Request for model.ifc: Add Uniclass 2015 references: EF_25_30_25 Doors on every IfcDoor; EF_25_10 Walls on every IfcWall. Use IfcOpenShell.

First a look at what the model holds.

```python
import ifcopenshell

model = ifcopenshell.open("model.ifc")
print(model.schema)
print("classifications:", [c.Name for c in model.by_type("IfcClassification")])
for ifc_class in ("IfcDoor", "IfcRoof", "IfcStair", "IfcWall", "IfcWindow"):
    print(ifc_class, len(model.by_type(ifc_class)))
```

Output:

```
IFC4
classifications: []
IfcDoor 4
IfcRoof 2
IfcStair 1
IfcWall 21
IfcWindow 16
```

```python
import ifcopenshell
import ifcopenshell.api.classification

model = ifcopenshell.open("model.ifc")

system = ifcopenshell.api.classification.add_classification(model, classification="Uniclass 2015")

codes = {
    "IfcDoor": ("EF_25_30_25", "Doors"),
    "IfcWall": ("EF_25_10", "Walls"),
}
for ifc_class, (code, name) in codes.items():
    products = model.by_type(ifc_class)
    ifcopenshell.api.classification.add_reference(
        model, products=products, classification=system, identification=code, name=name
    )
    print(code, len(products))

model.write("model_rev.ifc")
```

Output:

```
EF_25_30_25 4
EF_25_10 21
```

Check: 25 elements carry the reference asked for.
